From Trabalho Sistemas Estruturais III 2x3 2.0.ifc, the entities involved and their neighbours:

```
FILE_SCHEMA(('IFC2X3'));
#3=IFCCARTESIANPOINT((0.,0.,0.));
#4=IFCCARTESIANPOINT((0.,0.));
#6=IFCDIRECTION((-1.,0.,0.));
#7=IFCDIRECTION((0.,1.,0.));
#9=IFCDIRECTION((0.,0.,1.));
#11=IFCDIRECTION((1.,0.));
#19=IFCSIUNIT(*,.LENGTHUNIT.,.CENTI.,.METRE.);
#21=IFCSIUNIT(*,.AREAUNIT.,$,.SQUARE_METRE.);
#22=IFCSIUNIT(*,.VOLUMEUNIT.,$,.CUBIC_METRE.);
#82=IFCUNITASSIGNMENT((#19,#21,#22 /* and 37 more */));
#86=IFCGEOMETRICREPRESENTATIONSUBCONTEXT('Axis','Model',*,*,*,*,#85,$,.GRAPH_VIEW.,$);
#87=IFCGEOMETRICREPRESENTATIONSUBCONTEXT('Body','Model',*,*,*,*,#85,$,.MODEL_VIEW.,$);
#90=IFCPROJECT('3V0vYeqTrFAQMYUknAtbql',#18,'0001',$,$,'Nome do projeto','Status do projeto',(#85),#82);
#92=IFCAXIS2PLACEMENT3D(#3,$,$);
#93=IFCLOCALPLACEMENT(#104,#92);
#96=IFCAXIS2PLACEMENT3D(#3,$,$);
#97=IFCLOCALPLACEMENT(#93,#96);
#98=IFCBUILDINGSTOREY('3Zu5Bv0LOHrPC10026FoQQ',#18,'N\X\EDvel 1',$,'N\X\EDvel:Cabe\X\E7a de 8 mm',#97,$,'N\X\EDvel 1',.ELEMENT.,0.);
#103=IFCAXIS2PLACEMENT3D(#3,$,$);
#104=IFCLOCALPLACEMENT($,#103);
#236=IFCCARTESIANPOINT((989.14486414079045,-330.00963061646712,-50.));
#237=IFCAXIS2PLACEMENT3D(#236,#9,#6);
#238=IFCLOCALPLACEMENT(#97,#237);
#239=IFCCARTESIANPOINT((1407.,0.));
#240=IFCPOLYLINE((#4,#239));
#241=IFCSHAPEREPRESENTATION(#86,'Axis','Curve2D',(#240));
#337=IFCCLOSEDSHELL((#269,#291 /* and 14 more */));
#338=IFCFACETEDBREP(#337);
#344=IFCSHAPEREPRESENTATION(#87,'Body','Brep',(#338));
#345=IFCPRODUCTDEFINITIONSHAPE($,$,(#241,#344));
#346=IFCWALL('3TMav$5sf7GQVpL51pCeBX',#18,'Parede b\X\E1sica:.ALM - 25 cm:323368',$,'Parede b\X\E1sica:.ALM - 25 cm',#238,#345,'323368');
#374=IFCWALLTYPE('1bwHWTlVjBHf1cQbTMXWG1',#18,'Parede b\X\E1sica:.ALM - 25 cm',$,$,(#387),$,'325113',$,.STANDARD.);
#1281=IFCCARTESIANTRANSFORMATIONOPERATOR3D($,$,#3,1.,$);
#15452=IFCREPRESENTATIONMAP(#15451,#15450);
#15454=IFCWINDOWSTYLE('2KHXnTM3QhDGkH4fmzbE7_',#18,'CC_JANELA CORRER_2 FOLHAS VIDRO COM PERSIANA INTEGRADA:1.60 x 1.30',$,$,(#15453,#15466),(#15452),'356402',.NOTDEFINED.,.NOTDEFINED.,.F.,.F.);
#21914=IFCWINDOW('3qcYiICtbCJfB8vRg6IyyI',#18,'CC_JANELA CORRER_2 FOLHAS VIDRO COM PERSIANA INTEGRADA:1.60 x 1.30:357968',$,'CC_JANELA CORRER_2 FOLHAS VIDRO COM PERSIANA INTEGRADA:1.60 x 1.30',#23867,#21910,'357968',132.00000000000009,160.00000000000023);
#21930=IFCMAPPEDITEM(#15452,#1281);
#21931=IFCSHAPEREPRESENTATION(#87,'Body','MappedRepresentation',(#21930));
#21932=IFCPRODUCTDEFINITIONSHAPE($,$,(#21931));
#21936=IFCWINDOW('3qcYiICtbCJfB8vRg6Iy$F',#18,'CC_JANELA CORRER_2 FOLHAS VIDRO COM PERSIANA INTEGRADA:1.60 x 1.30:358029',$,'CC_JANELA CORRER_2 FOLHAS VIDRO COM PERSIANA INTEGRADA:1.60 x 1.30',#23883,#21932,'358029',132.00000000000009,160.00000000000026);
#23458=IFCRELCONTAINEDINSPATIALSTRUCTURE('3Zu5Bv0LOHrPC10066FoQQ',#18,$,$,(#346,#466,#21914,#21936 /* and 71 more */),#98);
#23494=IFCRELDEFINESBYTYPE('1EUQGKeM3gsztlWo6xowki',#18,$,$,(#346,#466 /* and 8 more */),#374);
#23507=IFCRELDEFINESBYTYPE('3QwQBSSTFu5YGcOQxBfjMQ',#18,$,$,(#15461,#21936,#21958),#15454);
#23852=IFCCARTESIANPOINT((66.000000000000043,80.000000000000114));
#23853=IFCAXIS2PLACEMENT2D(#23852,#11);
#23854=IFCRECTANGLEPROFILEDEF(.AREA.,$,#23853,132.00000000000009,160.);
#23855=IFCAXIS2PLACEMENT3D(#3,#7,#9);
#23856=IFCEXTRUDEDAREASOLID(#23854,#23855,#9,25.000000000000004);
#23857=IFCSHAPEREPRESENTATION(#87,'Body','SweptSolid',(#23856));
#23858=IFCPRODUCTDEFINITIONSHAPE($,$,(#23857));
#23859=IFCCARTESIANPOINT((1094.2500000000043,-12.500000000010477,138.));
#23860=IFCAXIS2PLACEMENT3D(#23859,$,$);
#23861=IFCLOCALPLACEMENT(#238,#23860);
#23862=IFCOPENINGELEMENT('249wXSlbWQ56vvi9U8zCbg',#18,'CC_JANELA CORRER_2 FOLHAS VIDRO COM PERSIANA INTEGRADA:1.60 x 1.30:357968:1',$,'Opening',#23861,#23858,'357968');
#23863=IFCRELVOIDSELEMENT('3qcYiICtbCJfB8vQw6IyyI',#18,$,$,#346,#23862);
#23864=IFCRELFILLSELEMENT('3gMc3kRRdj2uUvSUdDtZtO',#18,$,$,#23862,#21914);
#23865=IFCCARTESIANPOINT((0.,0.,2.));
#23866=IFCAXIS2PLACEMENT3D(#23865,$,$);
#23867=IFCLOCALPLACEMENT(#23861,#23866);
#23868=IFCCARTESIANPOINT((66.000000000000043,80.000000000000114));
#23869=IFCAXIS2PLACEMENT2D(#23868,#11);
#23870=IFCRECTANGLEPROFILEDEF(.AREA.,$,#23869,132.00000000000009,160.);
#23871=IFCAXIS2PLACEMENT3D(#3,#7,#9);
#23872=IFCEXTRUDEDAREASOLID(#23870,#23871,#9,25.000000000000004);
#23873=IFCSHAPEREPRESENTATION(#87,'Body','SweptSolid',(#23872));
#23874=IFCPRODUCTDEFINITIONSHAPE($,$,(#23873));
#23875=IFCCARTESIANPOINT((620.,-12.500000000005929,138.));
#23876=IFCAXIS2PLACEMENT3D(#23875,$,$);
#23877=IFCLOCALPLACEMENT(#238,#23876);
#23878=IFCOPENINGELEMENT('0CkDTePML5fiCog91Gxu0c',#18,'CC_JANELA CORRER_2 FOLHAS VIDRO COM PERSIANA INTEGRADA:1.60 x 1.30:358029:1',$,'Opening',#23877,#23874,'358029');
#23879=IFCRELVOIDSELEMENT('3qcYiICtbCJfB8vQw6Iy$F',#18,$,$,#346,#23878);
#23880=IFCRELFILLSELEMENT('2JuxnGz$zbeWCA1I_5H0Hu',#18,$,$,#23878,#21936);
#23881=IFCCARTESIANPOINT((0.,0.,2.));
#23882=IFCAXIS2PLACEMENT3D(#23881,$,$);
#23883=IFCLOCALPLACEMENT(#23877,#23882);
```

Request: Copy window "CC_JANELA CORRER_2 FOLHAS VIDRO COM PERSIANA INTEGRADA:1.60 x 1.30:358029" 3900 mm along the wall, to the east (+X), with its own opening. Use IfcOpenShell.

```python
import ifcopenshell
import ifcopenshell.api.feature
import ifcopenshell.api.geometry
import ifcopenshell.api.root
import ifcopenshell.geom
import ifcopenshell.util.element
import ifcopenshell.util.placement
import ifcopenshell.util.shape
import ifcopenshell.util.unit

model = ifcopenshell.open("Trabalho Sistemas Estruturais III 2x3 2.0.ifc")
unit_scale = ifcopenshell.util.unit.calculate_unit_scale(model)
settings = ifcopenshell.geom.settings()


def volume(element):
    """Net volume in cubic metres, openings subtracted."""
    shape = ifcopenshell.geom.create_shape(settings, element)
    return ifcopenshell.util.shape.get_volume(shape.geometry)


def reuse_history(source, copy):
    """copy_class also copies each property set's owner history, people and application; keep the originals."""
    for rel in copy.IsDefinedBy:
        if rel.is_a("IfcRelDefinesByProperties") and (history := rel.RelatingPropertyDefinition.OwnerHistory):
            rel.RelatingPropertyDefinition.OwnerHistory = source.OwnerHistory
            ifcopenshell.util.element.remove_deep2(model, history)


window = model.by_id(21936)
opening = window.FillsVoids[0].RelatingOpeningElement
wall = opening.VoidsElements[0].RelatingBuildingElement
before = volume(wall)
shift = ifcopenshell.util.placement.get_local_placement(wall.ObjectPlacement)[:3, 0] * -3.9 / unit_scale

# copy_class copies the void relationship, type, container and properties, but no geometry.
new_opening = ifcopenshell.api.root.copy_class(model, product=opening)
new_opening.Representation = ifcopenshell.util.element.copy_deep(
    model, opening.Representation, exclude=["IfcGeometricRepresentationContext", "IfcRepresentationMap"]
)
new_opening.Name = "CC_JANELA CORRER_2 FOLHAS VIDRO COM PERSIANA INTEGRADA:1.60 x 1.30"
new_opening.Tag = None
new_window = ifcopenshell.api.root.copy_class(model, product=window)
new_window.Representation = ifcopenshell.util.element.copy_deep(
    model, window.Representation, exclude=["IfcGeometricRepresentationContext", "IfcRepresentationMap"]
)
new_window.Name = "CC_JANELA CORRER_2 FOLHAS VIDRO COM PERSIANA INTEGRADA:1.60 x 1.30"
new_window.Tag = None
reuse_history(window, new_window)
fills = ifcopenshell.api.feature.add_filling(model, opening=new_opening, element=new_window)
fills.OwnerHistory = new_window.OwnerHistory  # required in IFC2X3

for old, new in ((opening, new_opening), (window, new_window)):
    matrix = ifcopenshell.util.placement.get_local_placement(old.ObjectPlacement)
    matrix[:3, 3] += shift
    ifcopenshell.api.geometry.edit_object_placement(model, product=new, matrix=matrix, is_si=False)

after = volume(wall)

print(f"wall volume {before:.3f} -> {after:.3f} m3")

model.write("Trabalho Sistemas Estruturais III 2x3 2.0_edited.ifc")
```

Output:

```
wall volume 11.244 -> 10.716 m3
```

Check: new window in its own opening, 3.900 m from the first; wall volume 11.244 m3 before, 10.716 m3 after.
